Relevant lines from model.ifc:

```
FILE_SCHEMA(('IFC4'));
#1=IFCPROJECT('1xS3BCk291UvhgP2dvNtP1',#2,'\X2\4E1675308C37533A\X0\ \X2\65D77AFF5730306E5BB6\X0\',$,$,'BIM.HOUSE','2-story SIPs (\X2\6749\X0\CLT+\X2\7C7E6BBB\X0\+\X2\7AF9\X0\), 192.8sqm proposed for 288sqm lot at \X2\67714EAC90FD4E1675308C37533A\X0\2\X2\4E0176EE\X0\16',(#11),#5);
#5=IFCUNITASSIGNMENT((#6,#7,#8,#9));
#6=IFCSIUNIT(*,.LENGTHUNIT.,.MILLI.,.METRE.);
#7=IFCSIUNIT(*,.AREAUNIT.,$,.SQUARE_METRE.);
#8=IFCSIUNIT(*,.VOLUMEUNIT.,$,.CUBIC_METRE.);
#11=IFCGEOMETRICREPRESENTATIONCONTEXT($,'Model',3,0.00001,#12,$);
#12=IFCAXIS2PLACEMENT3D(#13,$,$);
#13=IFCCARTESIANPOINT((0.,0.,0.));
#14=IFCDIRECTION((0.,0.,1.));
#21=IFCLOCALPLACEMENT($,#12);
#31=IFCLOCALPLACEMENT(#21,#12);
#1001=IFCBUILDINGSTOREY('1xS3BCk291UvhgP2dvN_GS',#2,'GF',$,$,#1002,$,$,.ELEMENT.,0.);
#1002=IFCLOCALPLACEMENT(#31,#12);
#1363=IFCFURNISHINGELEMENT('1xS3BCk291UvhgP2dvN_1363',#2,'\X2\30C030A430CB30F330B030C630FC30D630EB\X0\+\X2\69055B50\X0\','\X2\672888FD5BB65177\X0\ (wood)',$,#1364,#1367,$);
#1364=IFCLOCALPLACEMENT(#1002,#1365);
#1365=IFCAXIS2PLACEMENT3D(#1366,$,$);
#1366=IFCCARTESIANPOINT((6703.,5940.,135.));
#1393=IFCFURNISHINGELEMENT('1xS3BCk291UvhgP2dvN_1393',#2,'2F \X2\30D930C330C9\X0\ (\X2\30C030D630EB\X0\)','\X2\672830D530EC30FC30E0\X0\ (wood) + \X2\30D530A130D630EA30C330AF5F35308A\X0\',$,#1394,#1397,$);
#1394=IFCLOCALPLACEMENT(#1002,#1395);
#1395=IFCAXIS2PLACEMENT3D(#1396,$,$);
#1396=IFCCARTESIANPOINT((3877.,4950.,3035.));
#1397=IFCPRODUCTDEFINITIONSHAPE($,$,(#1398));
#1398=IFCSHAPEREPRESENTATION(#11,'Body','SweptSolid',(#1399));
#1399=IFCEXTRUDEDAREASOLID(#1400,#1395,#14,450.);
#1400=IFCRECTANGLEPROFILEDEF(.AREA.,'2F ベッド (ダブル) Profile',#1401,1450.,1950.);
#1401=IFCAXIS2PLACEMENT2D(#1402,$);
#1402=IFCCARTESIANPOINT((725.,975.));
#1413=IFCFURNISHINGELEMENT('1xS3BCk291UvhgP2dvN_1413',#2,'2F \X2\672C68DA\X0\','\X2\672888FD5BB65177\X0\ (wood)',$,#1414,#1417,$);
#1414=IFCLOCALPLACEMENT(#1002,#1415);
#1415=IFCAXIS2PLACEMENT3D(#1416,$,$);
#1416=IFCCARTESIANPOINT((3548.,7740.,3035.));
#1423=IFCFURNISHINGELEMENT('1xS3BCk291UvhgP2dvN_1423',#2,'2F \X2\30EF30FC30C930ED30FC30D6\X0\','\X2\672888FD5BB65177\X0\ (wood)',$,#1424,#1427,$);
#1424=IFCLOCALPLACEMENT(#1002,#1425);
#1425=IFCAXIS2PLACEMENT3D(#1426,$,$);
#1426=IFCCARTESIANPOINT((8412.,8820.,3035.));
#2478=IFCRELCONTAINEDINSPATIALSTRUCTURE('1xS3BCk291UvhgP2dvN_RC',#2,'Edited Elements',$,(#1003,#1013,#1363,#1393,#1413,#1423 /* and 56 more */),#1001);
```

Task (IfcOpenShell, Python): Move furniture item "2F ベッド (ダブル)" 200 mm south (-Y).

```python
import ifcopenshell
import ifcopenshell.api.geometry
import ifcopenshell.util.placement
import ifcopenshell.util.unit

model = ifcopenshell.open("model.ifc")
unit_scale = ifcopenshell.util.unit.calculate_unit_scale(model)

item = model.by_guid("1xS3BCk291UvhgP2dvN_1393")
matrix = ifcopenshell.util.placement.get_local_placement(item.ObjectPlacement)
matrix[1, 3] -= 0.2 / unit_scale
ifcopenshell.api.geometry.edit_object_placement(model, product=item, matrix=matrix, is_si=False)

print(ifcopenshell.util.placement.get_local_placement(item.ObjectPlacement).round(3) + 0.0)

model.write("model-out.ifc")
```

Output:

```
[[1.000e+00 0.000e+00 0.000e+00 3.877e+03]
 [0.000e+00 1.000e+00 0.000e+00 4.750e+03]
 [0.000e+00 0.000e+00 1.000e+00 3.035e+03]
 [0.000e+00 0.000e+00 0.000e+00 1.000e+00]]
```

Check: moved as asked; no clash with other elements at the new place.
